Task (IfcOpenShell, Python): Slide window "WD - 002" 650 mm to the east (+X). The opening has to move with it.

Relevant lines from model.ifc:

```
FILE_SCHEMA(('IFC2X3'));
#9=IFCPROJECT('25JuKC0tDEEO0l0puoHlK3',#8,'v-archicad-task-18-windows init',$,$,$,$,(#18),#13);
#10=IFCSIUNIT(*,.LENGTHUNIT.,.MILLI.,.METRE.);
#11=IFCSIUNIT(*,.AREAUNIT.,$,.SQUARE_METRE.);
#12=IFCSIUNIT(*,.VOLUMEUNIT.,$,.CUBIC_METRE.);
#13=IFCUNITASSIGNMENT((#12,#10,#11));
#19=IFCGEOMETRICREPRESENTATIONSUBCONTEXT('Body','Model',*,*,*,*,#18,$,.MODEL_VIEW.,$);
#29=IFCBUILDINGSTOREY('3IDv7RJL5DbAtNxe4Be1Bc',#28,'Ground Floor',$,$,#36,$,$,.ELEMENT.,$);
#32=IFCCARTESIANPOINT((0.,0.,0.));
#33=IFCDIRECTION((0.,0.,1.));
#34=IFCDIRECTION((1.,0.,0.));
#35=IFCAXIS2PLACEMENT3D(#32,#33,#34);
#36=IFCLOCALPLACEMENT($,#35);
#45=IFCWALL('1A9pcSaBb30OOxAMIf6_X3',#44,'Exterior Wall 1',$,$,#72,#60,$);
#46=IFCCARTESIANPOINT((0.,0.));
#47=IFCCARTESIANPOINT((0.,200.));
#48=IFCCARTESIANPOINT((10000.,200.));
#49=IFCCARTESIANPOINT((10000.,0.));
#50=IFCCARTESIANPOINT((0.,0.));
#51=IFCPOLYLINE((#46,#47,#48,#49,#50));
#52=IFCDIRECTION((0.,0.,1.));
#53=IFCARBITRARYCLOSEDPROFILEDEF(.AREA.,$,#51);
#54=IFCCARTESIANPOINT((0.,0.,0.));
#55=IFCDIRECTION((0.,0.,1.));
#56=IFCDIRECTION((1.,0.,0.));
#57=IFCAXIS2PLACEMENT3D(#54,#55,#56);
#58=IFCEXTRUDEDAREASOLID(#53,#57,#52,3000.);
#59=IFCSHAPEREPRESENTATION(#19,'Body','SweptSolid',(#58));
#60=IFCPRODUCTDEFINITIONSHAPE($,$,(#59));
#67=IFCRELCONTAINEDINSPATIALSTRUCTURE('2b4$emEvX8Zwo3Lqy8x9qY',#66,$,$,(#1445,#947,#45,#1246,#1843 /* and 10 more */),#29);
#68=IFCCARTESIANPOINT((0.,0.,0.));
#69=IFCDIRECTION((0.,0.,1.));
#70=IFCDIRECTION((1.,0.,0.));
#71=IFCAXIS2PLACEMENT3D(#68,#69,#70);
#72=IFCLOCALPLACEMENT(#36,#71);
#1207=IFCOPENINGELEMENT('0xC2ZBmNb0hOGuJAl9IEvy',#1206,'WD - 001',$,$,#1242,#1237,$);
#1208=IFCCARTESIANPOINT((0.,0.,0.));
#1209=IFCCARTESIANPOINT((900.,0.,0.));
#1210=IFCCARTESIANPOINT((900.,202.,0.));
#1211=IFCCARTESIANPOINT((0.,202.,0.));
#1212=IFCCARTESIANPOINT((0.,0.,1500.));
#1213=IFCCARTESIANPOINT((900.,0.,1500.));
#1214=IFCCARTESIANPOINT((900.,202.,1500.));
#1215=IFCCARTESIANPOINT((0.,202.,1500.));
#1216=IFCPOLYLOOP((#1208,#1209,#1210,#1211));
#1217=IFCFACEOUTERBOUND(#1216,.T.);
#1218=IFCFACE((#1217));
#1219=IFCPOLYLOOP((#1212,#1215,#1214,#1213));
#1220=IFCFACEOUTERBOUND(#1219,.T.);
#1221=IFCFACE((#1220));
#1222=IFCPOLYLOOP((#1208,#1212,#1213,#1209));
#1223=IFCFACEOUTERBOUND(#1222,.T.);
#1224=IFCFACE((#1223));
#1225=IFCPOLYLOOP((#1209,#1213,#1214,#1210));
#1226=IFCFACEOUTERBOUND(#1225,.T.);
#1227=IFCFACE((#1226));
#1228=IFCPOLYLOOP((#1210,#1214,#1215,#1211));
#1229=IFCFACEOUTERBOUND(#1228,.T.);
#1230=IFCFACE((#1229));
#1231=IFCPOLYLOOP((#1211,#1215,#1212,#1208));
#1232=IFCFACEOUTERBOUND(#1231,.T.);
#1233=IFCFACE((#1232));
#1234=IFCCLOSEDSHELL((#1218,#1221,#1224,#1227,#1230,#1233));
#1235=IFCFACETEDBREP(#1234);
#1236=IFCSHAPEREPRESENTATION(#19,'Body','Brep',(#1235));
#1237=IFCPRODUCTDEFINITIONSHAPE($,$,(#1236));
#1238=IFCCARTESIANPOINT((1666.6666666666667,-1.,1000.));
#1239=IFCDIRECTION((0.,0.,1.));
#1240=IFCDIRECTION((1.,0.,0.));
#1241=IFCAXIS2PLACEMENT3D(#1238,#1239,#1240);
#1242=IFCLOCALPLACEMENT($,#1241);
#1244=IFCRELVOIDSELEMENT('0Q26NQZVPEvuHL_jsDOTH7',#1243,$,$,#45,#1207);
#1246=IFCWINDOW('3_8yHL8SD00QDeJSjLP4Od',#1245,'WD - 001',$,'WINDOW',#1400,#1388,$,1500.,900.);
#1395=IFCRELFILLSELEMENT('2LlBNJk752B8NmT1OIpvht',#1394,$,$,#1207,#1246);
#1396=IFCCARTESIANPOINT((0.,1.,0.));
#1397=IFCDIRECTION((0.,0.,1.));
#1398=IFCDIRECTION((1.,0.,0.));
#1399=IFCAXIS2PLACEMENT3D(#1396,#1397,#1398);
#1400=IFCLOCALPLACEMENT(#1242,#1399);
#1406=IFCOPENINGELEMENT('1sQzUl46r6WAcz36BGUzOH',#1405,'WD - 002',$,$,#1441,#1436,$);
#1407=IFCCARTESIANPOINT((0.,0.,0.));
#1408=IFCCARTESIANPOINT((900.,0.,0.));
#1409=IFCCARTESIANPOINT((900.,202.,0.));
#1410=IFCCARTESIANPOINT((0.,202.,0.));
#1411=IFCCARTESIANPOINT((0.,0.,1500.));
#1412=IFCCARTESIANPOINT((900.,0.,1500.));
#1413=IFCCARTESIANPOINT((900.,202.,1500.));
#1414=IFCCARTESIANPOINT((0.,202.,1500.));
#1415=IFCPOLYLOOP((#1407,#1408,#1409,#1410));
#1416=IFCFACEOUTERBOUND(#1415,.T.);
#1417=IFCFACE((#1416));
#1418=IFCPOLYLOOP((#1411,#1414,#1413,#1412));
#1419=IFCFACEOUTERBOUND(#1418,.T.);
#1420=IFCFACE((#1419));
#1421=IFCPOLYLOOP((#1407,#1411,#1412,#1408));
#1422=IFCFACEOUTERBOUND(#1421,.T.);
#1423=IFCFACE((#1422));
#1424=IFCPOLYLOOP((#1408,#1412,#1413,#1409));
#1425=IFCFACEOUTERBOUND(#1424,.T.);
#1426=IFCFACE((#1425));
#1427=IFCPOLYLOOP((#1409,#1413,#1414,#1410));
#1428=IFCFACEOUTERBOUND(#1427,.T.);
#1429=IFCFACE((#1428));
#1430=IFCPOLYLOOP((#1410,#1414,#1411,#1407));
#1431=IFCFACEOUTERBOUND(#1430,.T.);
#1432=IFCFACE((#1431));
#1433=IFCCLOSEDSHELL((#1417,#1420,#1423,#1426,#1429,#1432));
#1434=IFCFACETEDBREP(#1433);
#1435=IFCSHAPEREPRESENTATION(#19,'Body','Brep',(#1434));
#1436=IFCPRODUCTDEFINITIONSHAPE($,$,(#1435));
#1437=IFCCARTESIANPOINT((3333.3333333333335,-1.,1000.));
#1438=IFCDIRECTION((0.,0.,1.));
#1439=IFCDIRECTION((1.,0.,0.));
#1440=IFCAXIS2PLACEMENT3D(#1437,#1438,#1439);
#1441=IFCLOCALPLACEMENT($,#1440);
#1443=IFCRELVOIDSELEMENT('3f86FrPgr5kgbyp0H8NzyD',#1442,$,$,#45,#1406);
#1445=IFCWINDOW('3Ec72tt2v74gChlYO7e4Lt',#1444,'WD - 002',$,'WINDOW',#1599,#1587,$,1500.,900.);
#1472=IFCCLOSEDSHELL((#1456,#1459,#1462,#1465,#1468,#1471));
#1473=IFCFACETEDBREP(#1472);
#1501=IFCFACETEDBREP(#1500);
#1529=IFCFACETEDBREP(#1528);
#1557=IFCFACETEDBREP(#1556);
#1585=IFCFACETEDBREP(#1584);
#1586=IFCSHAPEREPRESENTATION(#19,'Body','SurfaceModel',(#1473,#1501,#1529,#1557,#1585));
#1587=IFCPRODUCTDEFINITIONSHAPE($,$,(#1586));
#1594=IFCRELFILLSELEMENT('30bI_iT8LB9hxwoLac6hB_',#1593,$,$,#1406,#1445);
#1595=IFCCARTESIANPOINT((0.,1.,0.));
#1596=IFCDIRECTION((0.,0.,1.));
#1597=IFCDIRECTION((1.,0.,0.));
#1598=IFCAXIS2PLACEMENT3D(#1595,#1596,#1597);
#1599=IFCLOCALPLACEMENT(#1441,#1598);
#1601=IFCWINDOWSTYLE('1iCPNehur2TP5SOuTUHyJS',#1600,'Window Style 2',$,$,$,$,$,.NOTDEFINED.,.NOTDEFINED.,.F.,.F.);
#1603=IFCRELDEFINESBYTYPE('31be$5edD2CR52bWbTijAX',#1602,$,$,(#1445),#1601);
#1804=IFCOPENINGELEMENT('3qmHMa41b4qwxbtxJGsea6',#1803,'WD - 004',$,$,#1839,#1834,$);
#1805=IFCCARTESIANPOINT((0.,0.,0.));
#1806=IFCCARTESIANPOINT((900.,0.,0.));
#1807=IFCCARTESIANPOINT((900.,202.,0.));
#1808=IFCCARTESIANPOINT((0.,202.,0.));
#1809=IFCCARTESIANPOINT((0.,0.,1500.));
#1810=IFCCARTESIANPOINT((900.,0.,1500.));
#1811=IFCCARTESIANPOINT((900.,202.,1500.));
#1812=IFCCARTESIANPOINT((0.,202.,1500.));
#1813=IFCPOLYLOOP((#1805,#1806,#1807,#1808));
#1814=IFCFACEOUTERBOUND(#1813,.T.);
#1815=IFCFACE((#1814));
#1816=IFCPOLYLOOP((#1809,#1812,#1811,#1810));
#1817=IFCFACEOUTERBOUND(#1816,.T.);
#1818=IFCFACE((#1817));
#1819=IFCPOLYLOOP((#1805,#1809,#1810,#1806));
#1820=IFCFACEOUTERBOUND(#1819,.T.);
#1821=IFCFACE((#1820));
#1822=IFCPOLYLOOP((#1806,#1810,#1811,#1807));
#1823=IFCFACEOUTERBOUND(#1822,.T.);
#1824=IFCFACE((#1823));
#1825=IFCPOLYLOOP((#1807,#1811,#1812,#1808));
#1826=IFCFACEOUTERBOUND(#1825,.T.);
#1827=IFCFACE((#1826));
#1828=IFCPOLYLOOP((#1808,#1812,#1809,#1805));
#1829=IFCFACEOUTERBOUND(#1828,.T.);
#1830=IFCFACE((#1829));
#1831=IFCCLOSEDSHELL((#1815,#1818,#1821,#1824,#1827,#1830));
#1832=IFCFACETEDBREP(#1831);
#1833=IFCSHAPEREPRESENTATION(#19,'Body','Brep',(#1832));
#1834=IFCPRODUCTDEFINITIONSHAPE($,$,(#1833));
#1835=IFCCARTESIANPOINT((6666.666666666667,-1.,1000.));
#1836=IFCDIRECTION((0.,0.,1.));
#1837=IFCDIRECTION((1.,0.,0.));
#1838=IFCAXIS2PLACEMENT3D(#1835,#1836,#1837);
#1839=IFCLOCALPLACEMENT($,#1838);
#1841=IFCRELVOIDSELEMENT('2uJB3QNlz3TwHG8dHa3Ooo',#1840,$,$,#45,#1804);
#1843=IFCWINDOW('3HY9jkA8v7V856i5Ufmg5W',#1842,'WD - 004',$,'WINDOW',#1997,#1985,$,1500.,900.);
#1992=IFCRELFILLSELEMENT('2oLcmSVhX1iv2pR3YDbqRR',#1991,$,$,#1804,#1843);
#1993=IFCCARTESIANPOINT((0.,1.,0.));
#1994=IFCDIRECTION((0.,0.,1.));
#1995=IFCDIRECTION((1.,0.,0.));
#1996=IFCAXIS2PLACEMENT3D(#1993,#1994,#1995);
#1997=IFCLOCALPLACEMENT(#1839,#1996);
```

```python
import ifcopenshell
import ifcopenshell.api.geometry
import ifcopenshell.util.placement
import ifcopenshell.util.unit

model = ifcopenshell.open("model.ifc")
unit_scale = ifcopenshell.util.unit.calculate_unit_scale(model)

window = model.by_guid("3Ec72tt2v74gChlYO7e4Lt")
opening = window.FillsVoids[0].RelatingOpeningElement
wall = opening.VoidsElements[0].RelatingBuildingElement

wall_matrix = ifcopenshell.util.placement.get_local_placement(wall.ObjectPlacement)
shift = wall_matrix[:3, 0] * 0.65 / unit_scale
before = ifcopenshell.util.placement.get_local_placement(window.ObjectPlacement)[:3, 3].copy()

# The window is placed relative to its opening, so it follows when the opening moves.
matrix = ifcopenshell.util.placement.get_local_placement(opening.ObjectPlacement)
matrix[:3, 3] += shift
ifcopenshell.api.geometry.edit_object_placement(
    model, product=opening, matrix=matrix, is_si=False, should_transform_children=True
)

after = ifcopenshell.util.placement.get_local_placement(window.ObjectPlacement)[:3, 3]
print("window moved by", (after - before).round(3) + 0.0)

model.write("model_updated.ifc")
```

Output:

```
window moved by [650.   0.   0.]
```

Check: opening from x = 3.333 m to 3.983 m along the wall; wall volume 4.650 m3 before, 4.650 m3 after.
